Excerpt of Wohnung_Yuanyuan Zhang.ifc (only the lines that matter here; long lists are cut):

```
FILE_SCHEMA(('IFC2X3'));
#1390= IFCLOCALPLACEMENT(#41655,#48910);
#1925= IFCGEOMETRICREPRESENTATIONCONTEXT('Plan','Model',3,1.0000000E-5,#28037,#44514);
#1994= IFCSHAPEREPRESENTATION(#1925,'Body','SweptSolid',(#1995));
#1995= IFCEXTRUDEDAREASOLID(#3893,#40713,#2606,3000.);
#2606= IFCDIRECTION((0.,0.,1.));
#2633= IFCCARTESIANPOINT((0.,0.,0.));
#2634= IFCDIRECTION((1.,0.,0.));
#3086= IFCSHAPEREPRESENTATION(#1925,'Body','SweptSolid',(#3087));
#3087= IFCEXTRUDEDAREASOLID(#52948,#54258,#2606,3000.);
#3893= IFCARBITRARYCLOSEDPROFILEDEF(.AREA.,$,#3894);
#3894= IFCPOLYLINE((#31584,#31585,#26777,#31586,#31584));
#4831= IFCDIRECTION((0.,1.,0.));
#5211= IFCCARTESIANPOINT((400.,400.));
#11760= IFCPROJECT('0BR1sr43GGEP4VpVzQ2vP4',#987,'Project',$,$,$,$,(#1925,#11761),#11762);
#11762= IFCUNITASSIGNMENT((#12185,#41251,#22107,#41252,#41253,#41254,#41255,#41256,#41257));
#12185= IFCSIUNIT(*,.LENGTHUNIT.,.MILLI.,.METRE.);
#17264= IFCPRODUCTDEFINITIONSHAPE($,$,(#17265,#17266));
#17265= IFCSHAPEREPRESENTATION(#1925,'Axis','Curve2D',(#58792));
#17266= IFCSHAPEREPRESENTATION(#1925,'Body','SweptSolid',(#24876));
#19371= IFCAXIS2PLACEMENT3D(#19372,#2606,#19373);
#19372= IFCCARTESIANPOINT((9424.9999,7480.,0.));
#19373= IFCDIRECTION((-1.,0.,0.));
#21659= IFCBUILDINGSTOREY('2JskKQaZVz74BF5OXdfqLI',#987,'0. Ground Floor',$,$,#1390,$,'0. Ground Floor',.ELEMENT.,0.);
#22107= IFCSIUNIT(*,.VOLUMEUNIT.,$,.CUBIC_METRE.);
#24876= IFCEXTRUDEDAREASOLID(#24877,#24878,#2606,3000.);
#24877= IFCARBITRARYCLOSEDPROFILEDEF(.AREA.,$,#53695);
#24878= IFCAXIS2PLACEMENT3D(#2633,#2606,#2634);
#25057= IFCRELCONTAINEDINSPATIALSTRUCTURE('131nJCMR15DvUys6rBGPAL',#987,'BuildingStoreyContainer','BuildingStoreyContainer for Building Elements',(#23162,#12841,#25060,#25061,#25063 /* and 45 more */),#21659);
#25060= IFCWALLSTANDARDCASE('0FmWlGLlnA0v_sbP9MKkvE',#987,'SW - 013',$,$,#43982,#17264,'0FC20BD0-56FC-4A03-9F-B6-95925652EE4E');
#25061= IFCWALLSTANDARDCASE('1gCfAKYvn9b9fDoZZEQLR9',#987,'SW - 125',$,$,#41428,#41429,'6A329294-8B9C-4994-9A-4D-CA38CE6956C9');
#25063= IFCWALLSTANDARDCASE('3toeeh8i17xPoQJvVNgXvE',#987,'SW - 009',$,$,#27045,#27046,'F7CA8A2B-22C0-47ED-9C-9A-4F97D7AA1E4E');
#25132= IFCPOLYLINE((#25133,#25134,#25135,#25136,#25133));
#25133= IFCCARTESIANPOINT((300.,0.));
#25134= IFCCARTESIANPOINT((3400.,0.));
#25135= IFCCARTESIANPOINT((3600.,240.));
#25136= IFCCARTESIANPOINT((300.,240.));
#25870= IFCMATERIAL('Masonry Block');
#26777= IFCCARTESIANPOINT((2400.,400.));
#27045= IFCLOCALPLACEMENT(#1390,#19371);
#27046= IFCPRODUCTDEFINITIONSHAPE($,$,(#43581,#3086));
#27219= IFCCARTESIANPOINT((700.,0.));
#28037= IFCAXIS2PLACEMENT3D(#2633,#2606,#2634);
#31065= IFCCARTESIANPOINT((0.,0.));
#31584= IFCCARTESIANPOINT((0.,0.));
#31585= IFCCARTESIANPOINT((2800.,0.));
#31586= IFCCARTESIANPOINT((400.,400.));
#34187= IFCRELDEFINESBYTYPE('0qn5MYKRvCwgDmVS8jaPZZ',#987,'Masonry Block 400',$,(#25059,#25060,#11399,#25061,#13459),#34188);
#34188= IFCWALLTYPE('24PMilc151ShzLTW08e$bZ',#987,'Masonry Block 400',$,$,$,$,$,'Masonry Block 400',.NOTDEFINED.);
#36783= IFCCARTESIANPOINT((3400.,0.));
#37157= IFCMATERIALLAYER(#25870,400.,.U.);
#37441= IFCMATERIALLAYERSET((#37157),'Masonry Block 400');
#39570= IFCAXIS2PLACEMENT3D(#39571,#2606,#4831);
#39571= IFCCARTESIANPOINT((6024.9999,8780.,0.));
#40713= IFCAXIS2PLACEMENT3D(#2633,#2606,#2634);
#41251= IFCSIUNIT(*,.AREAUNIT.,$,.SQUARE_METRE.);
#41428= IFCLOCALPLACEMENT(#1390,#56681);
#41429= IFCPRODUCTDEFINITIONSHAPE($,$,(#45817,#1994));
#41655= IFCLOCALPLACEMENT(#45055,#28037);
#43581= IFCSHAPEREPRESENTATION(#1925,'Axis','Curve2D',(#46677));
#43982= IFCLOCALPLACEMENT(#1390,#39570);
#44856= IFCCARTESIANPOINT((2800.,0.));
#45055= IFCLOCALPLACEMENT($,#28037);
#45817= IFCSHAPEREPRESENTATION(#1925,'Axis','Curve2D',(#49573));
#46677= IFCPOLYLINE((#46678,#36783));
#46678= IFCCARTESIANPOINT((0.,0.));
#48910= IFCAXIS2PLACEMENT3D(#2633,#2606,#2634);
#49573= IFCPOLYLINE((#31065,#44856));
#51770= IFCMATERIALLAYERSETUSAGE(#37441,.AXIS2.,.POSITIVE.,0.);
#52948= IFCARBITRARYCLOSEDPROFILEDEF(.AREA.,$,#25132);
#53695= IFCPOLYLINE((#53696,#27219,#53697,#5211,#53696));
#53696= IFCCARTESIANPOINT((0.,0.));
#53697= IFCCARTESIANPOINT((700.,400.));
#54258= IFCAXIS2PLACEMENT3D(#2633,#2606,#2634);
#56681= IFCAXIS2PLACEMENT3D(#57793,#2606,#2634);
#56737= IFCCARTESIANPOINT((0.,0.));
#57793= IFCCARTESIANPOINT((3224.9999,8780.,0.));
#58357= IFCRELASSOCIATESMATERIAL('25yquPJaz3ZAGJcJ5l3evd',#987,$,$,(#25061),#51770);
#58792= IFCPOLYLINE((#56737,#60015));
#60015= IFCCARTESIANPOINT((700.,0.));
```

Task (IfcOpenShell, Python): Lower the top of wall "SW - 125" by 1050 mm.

```python
import ifcopenshell
import ifcopenshell.geom
import ifcopenshell.util.shape
import ifcopenshell.util.unit

model = ifcopenshell.open("Wohnung_Yuanyuan Zhang.ifc")
unit_scale = ifcopenshell.util.unit.calculate_unit_scale(model)
settings = ifcopenshell.geom.settings()


def volume(element):
    """Net volume in cubic metres, openings subtracted."""
    shape = ifcopenshell.geom.create_shape(settings, element)
    return ifcopenshell.util.shape.get_volume(shape.geometry)


wall = model.by_guid("1gCfAKYvn9b9fDoZZEQLR9")
before = volume(wall)

body = next(r for r in wall.Representation.Representations if r.RepresentationIdentifier == "Body")
solid = body.Items[0]
old_height = solid.Depth
solid.Depth -= 1.05 / unit_scale
after = volume(wall)

print(f"height {old_height:g} -> {solid.Depth:g}, volume {before:.3f} -> {after:.3f} m3")

model.write("Wohnung_Yuanyuan Zhang_updated.ifc")
```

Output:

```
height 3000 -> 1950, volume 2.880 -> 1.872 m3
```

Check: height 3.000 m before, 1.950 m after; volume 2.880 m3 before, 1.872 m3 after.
